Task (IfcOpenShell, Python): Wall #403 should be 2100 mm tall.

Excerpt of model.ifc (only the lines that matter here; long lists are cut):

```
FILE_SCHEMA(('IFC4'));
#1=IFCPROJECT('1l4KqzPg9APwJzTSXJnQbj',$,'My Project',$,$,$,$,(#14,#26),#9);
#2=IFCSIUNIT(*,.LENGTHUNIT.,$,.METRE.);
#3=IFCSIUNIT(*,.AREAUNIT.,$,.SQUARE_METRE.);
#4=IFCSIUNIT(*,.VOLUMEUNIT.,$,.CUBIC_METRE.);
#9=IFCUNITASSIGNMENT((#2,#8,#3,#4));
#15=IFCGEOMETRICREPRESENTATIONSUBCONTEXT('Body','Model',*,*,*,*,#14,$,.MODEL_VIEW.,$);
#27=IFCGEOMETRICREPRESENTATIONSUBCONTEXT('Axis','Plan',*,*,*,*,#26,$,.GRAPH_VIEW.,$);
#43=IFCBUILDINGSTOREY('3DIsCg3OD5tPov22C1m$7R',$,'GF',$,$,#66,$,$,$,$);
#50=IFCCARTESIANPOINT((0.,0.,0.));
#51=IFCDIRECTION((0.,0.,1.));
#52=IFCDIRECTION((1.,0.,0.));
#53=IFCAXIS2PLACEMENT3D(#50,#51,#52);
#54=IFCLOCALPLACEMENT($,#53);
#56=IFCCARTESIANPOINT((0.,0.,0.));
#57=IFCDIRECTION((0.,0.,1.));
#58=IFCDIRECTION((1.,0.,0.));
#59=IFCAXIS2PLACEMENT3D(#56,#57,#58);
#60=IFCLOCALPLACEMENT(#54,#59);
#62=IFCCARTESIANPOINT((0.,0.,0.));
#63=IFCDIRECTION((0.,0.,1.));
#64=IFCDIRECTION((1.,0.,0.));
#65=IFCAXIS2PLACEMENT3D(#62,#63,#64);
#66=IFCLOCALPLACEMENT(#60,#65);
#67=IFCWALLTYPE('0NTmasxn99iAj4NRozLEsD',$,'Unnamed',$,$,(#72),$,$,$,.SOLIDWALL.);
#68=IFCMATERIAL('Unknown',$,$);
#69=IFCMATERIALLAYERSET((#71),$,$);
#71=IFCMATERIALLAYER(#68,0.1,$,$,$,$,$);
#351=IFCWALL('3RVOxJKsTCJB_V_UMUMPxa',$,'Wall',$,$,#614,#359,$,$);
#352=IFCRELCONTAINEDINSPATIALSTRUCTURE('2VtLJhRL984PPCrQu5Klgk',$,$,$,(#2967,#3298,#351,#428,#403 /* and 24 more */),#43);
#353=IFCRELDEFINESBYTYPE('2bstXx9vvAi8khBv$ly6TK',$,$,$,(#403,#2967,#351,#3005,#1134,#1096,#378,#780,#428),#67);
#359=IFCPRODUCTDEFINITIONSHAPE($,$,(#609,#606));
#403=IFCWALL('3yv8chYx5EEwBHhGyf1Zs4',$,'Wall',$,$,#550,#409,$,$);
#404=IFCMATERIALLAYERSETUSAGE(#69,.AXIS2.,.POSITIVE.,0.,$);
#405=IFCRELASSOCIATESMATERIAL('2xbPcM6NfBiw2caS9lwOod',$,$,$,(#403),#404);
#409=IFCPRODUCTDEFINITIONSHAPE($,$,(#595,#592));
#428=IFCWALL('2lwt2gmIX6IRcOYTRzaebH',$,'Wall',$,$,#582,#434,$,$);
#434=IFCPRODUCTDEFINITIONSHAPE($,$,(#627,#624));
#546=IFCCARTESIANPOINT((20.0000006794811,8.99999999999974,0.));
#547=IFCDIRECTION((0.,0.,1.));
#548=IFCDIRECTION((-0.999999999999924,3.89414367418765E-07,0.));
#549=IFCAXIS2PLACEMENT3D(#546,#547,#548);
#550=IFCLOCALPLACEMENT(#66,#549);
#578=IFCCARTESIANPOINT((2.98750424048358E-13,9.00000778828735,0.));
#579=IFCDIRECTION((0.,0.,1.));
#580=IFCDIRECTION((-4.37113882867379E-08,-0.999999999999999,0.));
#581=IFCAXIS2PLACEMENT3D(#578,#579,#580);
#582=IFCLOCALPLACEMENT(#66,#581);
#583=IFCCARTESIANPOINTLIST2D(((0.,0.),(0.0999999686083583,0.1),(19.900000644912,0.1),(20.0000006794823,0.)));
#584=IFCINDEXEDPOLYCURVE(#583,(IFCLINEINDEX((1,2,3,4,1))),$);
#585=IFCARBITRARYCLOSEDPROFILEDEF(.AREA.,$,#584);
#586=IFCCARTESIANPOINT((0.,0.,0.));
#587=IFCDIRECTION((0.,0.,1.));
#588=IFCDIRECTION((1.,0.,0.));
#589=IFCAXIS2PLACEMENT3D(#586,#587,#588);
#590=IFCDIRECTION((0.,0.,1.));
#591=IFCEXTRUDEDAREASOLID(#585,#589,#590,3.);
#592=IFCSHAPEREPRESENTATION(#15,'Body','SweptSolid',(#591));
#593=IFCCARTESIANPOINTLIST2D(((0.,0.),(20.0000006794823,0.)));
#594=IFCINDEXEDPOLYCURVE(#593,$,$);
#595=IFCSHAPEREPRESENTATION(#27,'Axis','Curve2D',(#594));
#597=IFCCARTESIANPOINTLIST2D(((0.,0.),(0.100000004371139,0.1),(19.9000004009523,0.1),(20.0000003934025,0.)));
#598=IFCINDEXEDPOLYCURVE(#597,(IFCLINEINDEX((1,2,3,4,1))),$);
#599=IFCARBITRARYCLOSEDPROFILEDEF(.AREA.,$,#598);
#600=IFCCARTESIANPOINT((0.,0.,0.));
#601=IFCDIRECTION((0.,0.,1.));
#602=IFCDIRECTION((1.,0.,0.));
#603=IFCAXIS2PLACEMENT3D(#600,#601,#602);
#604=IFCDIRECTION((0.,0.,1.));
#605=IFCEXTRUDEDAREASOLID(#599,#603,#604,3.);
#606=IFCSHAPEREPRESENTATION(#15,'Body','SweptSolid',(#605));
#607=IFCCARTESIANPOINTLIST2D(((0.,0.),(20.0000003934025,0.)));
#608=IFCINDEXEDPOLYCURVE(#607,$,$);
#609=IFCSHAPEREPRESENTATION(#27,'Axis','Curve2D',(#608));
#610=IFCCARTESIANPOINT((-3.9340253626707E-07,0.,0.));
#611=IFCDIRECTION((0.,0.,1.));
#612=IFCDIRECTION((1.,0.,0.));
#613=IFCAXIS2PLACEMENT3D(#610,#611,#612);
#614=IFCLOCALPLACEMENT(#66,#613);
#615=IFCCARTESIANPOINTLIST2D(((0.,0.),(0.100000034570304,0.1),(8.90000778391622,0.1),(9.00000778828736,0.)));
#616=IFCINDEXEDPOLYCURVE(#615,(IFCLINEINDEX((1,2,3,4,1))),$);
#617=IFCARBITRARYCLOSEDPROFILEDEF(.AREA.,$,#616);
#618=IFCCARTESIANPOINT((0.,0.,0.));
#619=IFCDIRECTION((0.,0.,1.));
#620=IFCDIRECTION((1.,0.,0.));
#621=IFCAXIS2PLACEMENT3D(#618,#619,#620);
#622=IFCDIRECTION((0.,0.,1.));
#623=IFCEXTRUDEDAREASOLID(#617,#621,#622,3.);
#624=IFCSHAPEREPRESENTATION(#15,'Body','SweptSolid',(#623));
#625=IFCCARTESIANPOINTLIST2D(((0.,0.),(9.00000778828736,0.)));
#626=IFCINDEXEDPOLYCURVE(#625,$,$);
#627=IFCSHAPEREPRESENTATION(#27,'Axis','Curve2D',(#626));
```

```python
import ifcopenshell
import ifcopenshell.geom
import ifcopenshell.util.representation
import ifcopenshell.util.shape

model = ifcopenshell.open("model.ifc")
settings = ifcopenshell.geom.settings()


def volume(element):
    """Net volume in cubic metres, openings subtracted."""
    shape = ifcopenshell.geom.create_shape(settings, element)
    return ifcopenshell.util.shape.get_volume(shape.geometry)


wall = model.by_guid("3yv8chYx5EEwBHhGyf1Zs4")
before = volume(wall)

body = ifcopenshell.util.representation.get_representation(wall, "Model", "Body")
solid = body.Items[0]
old_height = solid.Depth
solid.Depth = 2.1
after = volume(wall)

print(f"height {old_height:g} -> {solid.Depth:g}, volume {before:.3f} -> {after:.3f} m3")

model.write("model_updated.ifc")
```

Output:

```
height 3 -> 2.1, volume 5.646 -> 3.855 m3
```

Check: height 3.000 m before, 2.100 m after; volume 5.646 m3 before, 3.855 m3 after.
